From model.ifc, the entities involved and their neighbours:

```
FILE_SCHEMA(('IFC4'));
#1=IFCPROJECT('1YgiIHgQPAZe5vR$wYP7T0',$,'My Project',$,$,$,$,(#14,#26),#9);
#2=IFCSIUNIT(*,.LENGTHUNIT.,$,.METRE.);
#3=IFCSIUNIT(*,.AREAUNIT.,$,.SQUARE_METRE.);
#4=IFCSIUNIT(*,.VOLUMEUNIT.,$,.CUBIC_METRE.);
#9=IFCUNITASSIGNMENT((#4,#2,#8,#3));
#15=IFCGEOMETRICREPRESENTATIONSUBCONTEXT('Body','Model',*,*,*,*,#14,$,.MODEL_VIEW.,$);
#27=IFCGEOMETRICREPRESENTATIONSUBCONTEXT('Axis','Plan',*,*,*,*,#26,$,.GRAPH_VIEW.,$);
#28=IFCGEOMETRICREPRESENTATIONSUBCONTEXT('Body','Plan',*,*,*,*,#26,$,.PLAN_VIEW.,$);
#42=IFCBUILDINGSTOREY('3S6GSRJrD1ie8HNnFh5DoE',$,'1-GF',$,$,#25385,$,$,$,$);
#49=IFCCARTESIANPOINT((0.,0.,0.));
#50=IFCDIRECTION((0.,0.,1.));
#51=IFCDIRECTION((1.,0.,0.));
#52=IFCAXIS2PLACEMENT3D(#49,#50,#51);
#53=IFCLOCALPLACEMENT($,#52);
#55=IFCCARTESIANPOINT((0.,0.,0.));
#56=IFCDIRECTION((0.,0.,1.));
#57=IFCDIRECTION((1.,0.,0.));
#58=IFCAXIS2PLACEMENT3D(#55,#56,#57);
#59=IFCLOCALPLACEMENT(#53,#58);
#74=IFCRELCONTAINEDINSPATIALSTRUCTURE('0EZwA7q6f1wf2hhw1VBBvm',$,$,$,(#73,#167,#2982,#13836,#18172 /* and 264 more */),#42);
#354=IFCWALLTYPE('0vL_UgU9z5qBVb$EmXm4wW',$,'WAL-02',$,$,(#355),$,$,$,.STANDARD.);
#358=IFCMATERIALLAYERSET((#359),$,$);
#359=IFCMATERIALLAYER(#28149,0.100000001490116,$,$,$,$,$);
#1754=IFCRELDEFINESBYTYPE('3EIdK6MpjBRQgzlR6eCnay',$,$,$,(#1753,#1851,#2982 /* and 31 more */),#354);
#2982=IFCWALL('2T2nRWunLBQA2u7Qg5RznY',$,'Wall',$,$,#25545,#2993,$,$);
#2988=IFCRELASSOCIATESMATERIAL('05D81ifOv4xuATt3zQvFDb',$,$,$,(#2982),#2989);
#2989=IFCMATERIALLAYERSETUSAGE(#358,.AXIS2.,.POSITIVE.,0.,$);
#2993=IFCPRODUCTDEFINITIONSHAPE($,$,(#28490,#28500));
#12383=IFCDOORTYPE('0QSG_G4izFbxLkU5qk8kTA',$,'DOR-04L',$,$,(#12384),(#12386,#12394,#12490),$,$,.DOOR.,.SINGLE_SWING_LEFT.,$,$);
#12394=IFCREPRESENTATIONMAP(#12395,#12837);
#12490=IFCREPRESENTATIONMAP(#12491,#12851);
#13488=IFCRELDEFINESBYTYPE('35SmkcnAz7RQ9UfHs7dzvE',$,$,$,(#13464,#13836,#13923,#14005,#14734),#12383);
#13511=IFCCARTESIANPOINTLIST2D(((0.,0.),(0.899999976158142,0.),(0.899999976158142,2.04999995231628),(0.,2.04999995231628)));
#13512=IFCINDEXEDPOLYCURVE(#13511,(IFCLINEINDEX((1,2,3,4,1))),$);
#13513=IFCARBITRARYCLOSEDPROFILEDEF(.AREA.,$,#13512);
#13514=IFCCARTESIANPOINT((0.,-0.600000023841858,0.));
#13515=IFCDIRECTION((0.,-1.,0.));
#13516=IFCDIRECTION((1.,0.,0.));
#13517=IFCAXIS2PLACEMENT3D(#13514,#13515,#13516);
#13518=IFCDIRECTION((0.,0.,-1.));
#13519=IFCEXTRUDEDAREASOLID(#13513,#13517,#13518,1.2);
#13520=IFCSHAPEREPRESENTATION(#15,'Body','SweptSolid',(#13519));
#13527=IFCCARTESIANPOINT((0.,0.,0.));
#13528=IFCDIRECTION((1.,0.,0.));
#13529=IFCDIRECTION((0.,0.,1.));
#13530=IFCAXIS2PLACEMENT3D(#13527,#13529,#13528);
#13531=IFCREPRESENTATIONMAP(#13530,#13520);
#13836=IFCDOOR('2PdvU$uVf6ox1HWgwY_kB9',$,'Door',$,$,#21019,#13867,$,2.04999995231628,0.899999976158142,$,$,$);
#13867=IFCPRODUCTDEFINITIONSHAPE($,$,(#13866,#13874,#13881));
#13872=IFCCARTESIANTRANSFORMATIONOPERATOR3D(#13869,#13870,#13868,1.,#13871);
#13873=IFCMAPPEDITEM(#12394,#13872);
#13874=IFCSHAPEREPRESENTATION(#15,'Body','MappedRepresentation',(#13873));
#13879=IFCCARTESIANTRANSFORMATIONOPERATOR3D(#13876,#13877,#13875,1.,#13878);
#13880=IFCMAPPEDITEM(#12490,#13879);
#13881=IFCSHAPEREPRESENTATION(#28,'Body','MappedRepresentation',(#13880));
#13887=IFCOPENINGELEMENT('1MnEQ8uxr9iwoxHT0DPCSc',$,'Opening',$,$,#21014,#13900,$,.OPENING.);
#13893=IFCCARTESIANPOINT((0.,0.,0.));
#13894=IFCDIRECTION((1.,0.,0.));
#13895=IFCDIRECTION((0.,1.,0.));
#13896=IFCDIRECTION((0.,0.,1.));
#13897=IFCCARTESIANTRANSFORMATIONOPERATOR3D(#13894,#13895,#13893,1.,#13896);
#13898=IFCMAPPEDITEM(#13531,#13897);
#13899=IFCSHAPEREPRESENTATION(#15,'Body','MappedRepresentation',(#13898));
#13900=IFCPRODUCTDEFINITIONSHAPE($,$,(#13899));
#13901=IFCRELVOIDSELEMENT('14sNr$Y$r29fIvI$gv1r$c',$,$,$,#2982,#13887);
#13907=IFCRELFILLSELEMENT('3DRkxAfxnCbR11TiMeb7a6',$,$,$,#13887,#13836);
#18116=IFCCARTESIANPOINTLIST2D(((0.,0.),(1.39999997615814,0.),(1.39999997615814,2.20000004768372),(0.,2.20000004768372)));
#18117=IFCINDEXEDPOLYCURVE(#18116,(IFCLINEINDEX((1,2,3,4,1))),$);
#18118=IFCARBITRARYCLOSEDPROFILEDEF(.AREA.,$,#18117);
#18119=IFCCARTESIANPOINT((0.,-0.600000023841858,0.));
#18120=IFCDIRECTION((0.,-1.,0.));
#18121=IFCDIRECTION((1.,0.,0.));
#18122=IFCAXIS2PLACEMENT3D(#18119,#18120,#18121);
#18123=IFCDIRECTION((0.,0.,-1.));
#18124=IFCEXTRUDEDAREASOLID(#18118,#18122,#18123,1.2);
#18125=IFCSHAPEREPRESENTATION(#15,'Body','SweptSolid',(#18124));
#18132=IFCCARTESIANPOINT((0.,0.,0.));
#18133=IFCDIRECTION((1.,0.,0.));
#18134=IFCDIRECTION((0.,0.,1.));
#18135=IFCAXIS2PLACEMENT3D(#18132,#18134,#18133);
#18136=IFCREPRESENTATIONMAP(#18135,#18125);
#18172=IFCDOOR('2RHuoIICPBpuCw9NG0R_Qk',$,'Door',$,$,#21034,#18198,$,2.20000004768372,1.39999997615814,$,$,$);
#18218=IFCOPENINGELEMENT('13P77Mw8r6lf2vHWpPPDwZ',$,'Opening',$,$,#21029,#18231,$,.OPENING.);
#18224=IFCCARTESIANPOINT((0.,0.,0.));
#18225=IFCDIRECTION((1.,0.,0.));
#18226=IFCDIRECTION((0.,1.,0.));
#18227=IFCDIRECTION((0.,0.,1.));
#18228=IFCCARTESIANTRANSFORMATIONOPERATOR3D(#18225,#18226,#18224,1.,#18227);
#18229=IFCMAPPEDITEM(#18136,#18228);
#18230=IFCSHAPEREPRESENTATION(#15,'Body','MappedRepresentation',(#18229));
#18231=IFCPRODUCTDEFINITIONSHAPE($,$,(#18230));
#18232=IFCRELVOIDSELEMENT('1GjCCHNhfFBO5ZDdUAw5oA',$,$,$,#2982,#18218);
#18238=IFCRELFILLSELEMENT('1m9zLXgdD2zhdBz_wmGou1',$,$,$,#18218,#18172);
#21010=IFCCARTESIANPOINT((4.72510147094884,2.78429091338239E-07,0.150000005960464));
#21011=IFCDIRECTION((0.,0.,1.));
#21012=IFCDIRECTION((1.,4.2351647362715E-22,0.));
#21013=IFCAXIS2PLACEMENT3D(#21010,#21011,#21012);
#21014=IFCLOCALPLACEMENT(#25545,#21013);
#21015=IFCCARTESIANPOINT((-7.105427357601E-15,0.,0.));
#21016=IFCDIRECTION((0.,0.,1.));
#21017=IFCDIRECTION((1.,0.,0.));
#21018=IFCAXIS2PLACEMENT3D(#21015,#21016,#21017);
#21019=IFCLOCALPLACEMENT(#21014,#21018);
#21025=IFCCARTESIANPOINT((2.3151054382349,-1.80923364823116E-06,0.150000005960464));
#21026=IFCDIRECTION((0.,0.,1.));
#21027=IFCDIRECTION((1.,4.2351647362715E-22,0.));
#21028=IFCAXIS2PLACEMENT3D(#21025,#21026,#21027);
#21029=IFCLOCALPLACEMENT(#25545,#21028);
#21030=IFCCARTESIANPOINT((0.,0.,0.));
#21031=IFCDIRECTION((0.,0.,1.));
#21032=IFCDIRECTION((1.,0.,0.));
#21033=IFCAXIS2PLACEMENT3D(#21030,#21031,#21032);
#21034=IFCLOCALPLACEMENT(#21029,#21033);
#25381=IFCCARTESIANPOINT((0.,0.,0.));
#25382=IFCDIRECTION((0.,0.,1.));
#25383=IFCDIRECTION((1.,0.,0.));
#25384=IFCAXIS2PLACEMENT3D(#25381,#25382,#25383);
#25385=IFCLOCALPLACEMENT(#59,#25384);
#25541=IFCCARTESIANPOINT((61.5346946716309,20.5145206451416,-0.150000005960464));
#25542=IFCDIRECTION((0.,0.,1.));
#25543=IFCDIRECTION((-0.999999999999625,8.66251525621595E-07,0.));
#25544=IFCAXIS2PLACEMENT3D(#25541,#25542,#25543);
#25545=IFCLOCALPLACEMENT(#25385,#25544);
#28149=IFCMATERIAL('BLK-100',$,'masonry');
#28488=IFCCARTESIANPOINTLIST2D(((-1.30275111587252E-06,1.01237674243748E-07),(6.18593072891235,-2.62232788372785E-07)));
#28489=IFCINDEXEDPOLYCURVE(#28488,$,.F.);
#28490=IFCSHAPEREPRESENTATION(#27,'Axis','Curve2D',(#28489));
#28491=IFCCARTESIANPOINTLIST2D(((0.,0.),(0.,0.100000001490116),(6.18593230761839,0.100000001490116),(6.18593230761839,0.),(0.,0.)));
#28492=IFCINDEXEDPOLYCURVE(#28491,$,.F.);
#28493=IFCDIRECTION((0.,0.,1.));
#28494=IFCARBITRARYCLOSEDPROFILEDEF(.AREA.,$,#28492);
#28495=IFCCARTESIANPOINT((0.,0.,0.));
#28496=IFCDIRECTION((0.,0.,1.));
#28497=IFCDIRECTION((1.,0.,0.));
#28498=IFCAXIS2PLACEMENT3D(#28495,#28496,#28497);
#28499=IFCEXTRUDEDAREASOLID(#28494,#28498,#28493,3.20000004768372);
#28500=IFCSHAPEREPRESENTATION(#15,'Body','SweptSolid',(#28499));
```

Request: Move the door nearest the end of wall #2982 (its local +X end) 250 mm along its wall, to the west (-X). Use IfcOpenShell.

```python
import ifcopenshell
import ifcopenshell.api.geometry
import ifcopenshell.util.placement

model = ifcopenshell.open("model.ifc")

door = model.by_guid("2PdvU$uVf6ox1HWgwY_kB9")
opening = door.FillsVoids[0].RelatingOpeningElement
wall = opening.VoidsElements[0].RelatingBuildingElement

wall_matrix = ifcopenshell.util.placement.get_local_placement(wall.ObjectPlacement)
shift = wall_matrix[:3, 0] * 0.25
before = ifcopenshell.util.placement.get_local_placement(door.ObjectPlacement)[:3, 3].copy()

# The door is placed relative to its opening, so it follows when the opening moves.
matrix = ifcopenshell.util.placement.get_local_placement(opening.ObjectPlacement)
matrix[:3, 3] += shift
ifcopenshell.api.geometry.edit_object_placement(
    model, product=opening, matrix=matrix, is_si=False, should_transform_children=True
)

after = ifcopenshell.util.placement.get_local_placement(door.ObjectPlacement)[:3, 3]
print("door moved by", (after - before).round(3) + 0.0)

model.write("model_updated.ifc")
```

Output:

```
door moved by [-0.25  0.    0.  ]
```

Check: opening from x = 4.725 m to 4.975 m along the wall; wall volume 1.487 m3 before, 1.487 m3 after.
